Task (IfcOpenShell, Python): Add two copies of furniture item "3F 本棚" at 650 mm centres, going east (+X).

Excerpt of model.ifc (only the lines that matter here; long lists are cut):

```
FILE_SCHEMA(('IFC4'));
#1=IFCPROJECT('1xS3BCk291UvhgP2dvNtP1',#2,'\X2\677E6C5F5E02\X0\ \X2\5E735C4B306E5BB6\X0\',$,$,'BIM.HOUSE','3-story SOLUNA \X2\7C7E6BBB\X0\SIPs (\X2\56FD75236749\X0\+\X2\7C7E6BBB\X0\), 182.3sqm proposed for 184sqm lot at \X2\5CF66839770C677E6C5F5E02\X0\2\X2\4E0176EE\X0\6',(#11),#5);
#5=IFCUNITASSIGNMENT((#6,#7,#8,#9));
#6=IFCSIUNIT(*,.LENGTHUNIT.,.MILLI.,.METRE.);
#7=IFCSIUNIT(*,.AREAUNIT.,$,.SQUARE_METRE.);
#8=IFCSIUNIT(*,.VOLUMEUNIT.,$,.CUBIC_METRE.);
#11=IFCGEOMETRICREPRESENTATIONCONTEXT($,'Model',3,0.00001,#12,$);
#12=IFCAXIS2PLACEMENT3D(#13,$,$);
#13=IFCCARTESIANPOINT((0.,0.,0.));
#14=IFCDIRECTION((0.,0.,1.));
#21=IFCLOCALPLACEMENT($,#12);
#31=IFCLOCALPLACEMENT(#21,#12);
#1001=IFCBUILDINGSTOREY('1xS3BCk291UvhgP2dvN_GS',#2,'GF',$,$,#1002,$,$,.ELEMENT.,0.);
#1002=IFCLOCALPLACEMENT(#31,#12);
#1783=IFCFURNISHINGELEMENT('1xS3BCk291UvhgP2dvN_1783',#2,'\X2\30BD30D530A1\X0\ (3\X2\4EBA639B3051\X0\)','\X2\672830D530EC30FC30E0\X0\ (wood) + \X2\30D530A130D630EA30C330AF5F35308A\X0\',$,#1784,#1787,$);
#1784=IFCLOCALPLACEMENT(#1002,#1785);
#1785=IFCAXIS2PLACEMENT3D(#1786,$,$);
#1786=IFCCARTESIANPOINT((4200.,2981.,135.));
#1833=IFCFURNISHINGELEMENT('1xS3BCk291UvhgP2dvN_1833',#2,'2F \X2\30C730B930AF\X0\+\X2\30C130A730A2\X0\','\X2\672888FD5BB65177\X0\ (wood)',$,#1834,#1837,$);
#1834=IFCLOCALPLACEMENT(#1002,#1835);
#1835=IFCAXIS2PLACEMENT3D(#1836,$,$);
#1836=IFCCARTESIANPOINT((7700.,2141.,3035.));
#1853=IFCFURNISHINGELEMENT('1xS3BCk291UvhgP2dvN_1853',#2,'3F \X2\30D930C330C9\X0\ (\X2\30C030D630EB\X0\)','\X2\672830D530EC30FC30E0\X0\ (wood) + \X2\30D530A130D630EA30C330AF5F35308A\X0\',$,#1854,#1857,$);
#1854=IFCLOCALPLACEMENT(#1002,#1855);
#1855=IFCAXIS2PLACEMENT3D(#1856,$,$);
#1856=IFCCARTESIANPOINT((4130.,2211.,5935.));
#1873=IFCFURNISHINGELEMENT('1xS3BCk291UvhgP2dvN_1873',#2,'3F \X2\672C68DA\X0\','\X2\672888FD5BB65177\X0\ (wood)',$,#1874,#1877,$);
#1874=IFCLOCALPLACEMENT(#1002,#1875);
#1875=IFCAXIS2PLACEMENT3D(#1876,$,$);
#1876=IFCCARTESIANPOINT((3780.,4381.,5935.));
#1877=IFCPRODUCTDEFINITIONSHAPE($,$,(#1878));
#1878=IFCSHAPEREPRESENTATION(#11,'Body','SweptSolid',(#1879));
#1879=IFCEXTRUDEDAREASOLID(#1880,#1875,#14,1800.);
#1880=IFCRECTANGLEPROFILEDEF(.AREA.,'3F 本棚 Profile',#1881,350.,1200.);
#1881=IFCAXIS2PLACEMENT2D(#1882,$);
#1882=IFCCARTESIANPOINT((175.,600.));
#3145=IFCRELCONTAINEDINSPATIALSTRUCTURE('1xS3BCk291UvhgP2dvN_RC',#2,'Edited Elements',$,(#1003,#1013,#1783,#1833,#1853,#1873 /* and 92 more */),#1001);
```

```python
import numpy as np
import ifcopenshell
import ifcopenshell.api.geometry
import ifcopenshell.api.root
import ifcopenshell.util.element
import ifcopenshell.util.placement

model = ifcopenshell.open("model.ifc")


def reuse_history(source, copy):
    """copy_class also copies each property set's owner history, people and application; keep the originals."""
    for rel in copy.IsDefinedBy:
        if rel.is_a("IfcRelDefinesByProperties") and (history := rel.RelatingPropertyDefinition.OwnerHistory):
            rel.RelatingPropertyDefinition.OwnerHistory = source.OwnerHistory
            ifcopenshell.util.element.remove_deep2(model, history)


source = model.by_id(1873)
base = ifcopenshell.util.placement.get_local_placement(source.ObjectPlacement)
step = np.array([1.0, 0.0, 0.0]) * 650.0

for i in range(1, 3):
    copy = ifcopenshell.api.root.copy_class(model, product=source)
    copy.Representation = ifcopenshell.util.element.copy_deep(
        model, source.Representation, exclude=["IfcGeometricRepresentationContext", "IfcRepresentationMap"]
    )
    reuse_history(source, copy)
    matrix = base.copy()
    matrix[:3, 3] += i * step
    print("added at", matrix[:3, 3].round(3) + 0.0)
    ifcopenshell.api.geometry.edit_object_placement(model, product=copy, matrix=matrix, is_si=False)

model.write("model_edited.ifc")
```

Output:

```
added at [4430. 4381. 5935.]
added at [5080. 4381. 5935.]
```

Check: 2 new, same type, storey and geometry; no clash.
